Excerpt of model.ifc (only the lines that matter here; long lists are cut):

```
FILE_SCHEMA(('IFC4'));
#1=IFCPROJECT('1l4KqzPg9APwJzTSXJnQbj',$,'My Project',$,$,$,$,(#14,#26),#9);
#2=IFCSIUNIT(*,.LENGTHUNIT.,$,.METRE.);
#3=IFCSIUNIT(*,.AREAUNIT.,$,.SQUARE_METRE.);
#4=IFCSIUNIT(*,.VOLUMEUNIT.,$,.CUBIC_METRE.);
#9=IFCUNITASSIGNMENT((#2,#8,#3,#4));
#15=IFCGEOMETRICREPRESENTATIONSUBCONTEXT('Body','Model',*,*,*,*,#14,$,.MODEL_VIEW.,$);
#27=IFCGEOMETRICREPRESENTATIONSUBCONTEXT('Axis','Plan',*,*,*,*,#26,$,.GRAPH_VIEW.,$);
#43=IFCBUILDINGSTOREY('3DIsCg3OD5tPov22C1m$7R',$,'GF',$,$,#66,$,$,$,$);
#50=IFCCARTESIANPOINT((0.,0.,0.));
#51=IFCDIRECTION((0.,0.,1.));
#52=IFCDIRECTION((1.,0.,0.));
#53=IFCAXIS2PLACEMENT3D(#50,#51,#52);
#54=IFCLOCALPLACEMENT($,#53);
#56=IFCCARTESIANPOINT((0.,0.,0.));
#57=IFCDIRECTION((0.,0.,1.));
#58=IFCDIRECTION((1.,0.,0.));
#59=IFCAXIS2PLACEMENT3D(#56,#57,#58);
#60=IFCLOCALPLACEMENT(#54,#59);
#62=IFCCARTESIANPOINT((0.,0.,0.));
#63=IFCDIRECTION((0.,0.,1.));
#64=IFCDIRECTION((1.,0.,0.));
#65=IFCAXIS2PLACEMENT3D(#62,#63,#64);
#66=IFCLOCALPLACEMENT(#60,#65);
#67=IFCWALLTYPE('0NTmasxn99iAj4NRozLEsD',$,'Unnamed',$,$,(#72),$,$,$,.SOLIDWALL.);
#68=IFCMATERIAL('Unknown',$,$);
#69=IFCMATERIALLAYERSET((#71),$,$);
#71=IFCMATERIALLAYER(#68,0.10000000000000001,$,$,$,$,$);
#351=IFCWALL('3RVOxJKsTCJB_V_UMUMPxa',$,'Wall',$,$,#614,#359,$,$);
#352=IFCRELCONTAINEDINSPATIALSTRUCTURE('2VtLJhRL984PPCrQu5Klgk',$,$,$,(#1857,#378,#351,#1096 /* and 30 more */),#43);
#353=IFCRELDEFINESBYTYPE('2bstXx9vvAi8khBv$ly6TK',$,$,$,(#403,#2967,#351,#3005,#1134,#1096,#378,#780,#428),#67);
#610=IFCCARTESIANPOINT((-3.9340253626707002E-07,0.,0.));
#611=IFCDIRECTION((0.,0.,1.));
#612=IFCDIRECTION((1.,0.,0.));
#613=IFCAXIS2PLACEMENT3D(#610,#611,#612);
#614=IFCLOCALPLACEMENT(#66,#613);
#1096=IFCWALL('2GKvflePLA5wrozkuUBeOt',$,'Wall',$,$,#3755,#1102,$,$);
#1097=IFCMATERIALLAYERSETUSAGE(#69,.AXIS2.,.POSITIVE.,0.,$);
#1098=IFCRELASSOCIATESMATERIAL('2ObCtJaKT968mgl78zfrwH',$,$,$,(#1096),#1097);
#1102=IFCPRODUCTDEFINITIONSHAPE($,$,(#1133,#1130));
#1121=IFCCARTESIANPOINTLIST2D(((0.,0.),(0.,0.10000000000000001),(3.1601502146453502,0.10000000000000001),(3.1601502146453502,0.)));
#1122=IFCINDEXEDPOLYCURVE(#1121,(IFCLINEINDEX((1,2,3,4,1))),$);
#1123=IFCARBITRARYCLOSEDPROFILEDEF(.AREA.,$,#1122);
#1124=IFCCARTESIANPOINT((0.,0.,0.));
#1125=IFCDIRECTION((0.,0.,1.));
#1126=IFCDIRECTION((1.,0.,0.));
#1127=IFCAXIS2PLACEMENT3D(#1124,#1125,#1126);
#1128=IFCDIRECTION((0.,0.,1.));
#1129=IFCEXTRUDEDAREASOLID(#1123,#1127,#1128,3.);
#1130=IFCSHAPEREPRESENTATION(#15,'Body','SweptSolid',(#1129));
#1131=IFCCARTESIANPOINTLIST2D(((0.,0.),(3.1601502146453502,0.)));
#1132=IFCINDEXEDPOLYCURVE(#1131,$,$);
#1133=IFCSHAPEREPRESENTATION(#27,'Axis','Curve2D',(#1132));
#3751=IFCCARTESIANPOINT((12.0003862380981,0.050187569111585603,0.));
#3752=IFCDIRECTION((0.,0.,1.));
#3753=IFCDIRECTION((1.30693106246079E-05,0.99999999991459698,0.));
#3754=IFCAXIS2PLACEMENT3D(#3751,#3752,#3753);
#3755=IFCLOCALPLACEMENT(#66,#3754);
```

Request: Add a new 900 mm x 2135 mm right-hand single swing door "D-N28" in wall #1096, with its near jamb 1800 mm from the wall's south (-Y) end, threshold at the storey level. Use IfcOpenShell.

```python
import numpy as np
import ifcopenshell
import ifcopenshell.api.feature
import ifcopenshell.api.geometry
import ifcopenshell.api.root
import ifcopenshell.api.spatial
import ifcopenshell.geom
import ifcopenshell.util.element
import ifcopenshell.util.placement
import ifcopenshell.util.representation
import ifcopenshell.util.shape
import ifcopenshell.util.unit

model = ifcopenshell.open("model.ifc")
unit_scale = ifcopenshell.util.unit.calculate_unit_scale(model)
settings = ifcopenshell.geom.settings()


def volume(element):
    """Net volume in cubic metres, openings subtracted."""
    shape = ifcopenshell.geom.create_shape(settings, element)
    return ifcopenshell.util.shape.get_volume(shape.geometry)


wall = model.by_guid("2GKvflePLA5wrozkuUBeOt")
storey = ifcopenshell.util.element.get_container(wall, ifc_class="IfcBuildingStorey")
context = ifcopenshell.util.representation.get_context(model, "Model", "Body", "MODEL_VIEW")
before = volume(wall)

width, height, from_end, sill = 0.9, 2.135, 1.8, 0.0  # metres

# The wall runs along its own X axis, and the end named is its -X end.
wall_shape = ifcopenshell.geom.create_shape(settings, wall)
x, y, z = ifcopenshell.util.shape.get_vertices(wall_shape.geometry).T
start = x.min() + from_end
face, thickness = float(y.min()), float(y.max() - y.min())
wall_matrix = ifcopenshell.util.placement.get_local_placement(wall.ObjectPlacement)
level = ifcopenshell.util.placement.get_local_placement(storey.ObjectPlacement)[2, 3]


def in_wall(x, y):
    """Placement at x, y metres in the wall's axes, at sill height."""
    matrix = wall_matrix.copy()
    matrix[:, 3] = wall_matrix @ np.array([x / unit_scale, y / unit_scale, 0.0, 1.0])
    matrix[2, 3] = level + sill / unit_scale
    return matrix


# Opening: a box that overshoots both wall faces by 50 mm.
opening = ifcopenshell.api.root.create_entity(model, ifc_class="IfcOpeningElement", predefined_type="OPENING")
box = ifcopenshell.api.geometry.add_wall_representation(
    model, context=context, length=width, height=height, thickness=thickness + 0.1
)
ifcopenshell.api.geometry.assign_representation(model, product=opening, representation=box)
ifcopenshell.api.geometry.edit_object_placement(model, product=opening, matrix=in_wall(start, face - 0.05), is_si=False)
ifcopenshell.api.feature.add_feature(model, feature=opening, element=wall)

door = ifcopenshell.api.root.create_entity(model, ifc_class="IfcDoor", name="D-N28", predefined_type="DOOR")
door.OverallWidth, door.OverallHeight = width / unit_scale, height / unit_scale
door.OperationType = "SINGLE_SWING_RIGHT"
body = ifcopenshell.api.geometry.add_door_representation(
    model,
    context=context,
    overall_width=door.OverallWidth,
    overall_height=door.OverallHeight,
    operation_type="SINGLE_SWING_RIGHT",
    lining_properties={"LiningDepth": thickness / unit_scale, "ThresholdDepth": thickness / unit_scale},
)
ifcopenshell.api.geometry.assign_representation(model, product=door, representation=body)
ifcopenshell.api.spatial.assign_container(model, products=[door], relating_structure=storey)
ifcopenshell.api.feature.add_filling(model, opening=opening, element=door)

# The lining spans the wall, so the door starts at the wall face.
ifcopenshell.api.geometry.edit_object_placement(model, product=door, matrix=in_wall(start, face), is_si=False)

after = volume(wall)

print(f"wall volume {before:.3f} -> {after:.3f} m3")

model.write("model_edited.ifc")
```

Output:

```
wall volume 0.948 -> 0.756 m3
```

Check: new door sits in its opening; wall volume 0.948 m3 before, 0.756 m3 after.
